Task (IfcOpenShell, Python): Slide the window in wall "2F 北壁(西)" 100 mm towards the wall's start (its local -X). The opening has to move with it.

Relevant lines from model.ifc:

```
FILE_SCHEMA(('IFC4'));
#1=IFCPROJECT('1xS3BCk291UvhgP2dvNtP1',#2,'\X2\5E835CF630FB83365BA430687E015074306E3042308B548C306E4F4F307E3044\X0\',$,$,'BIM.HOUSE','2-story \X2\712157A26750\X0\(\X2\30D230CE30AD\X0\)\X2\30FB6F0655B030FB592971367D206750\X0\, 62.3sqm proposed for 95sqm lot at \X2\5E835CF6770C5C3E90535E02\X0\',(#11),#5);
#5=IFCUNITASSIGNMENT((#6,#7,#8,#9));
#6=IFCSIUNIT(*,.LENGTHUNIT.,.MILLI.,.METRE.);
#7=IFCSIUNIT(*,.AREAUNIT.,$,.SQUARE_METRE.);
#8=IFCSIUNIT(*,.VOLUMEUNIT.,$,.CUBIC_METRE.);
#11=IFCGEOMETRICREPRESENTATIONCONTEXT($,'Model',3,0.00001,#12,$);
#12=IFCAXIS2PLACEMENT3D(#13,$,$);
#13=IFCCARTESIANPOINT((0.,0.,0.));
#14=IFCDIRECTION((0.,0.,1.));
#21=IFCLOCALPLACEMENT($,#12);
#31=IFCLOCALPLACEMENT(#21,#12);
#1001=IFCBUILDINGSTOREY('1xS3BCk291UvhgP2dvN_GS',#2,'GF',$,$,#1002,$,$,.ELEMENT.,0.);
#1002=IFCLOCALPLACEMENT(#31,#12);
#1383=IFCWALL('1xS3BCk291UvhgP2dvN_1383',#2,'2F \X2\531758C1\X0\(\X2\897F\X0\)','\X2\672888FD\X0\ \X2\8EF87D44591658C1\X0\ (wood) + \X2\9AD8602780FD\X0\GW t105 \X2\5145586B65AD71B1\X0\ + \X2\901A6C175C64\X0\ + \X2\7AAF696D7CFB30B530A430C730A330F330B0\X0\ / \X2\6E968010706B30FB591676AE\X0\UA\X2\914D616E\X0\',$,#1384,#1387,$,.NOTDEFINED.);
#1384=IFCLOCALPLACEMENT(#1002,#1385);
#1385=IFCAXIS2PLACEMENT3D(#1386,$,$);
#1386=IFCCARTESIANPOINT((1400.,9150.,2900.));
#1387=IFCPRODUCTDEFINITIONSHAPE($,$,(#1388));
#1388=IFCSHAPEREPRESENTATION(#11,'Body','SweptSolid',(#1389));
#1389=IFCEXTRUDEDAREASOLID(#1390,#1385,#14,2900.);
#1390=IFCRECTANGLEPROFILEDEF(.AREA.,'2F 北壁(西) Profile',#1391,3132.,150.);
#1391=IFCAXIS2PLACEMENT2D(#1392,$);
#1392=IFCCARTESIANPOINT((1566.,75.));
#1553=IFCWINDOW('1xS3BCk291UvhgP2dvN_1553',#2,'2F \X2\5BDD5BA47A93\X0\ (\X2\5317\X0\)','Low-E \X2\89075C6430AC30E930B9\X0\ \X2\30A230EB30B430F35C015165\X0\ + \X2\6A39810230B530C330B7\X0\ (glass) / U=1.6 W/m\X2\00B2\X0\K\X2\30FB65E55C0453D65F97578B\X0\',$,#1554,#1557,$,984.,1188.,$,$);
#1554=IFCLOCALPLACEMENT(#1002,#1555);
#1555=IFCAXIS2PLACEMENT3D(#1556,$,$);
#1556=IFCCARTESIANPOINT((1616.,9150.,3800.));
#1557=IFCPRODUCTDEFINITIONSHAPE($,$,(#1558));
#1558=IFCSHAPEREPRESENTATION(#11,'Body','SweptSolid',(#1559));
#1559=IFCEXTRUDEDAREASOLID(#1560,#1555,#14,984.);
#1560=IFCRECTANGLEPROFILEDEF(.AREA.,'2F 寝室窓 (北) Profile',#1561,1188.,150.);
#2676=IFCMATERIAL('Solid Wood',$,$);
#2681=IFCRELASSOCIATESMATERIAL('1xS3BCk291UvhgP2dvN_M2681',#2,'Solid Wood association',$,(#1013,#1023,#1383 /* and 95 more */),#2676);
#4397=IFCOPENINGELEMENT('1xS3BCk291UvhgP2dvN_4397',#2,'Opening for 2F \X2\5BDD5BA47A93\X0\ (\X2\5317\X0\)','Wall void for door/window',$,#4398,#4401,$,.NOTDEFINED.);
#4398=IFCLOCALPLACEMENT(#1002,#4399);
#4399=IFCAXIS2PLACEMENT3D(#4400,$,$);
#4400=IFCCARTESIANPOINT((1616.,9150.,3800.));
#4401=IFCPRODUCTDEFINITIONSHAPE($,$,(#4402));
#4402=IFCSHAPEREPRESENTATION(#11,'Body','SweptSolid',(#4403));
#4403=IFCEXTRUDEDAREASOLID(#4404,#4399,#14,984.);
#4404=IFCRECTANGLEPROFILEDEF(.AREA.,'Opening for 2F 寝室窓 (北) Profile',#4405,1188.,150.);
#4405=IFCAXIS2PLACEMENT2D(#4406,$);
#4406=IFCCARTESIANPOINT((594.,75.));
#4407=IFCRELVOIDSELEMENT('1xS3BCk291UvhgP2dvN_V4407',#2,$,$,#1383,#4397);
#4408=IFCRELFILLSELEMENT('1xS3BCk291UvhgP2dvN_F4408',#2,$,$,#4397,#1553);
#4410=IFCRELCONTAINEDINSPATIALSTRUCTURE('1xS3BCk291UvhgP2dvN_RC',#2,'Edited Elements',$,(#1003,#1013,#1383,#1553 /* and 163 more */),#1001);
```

```python
import ifcopenshell
import ifcopenshell.api.geometry
import ifcopenshell.util.placement
import ifcopenshell.util.unit

model = ifcopenshell.open("model.ifc")
unit_scale = ifcopenshell.util.unit.calculate_unit_scale(model)

window = model.by_guid("1xS3BCk291UvhgP2dvN_1553")
opening = window.FillsVoids[0].RelatingOpeningElement
wall = opening.VoidsElements[0].RelatingBuildingElement

wall_matrix = ifcopenshell.util.placement.get_local_placement(wall.ObjectPlacement)
shift = wall_matrix[:3, 0] * -0.1 / unit_scale
before = ifcopenshell.util.placement.get_local_placement(window.ObjectPlacement)[:3, 3].copy()

# The window is not placed relative to its opening, so move both.
for product in (opening, window):
    matrix = ifcopenshell.util.placement.get_local_placement(product.ObjectPlacement)
    matrix[:3, 3] += shift
    ifcopenshell.api.geometry.edit_object_placement(model, product=product, matrix=matrix, is_si=False)

after = ifcopenshell.util.placement.get_local_placement(window.ObjectPlacement)[:3, 3]
print("window moved by", (after - before).round(3) + 0.0)

model.write("model_rev.ifc")
```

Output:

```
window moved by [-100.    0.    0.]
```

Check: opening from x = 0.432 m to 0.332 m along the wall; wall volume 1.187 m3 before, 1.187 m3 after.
